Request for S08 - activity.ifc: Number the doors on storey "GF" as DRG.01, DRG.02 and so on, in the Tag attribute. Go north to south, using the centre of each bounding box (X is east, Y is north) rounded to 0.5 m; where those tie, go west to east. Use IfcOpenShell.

First a look at what the model holds.

```python
import ifcopenshell
import ifcopenshell.util.element
import ifcopenshell.util.placement

model = ifcopenshell.open("S08 - activity.ifc")
print(model.schema)
storey = next(s for s in model.by_type("IfcBuildingStorey") if s.Name == "GF")
doors = [e for e in ifcopenshell.util.element.get_decomposition(storey) if e.is_a("IfcDoor")]
for e in sorted(doors, key=lambda e: e.id()):
    origin = ifcopenshell.util.placement.get_local_placement(e.ObjectPlacement)[:3, 3]
    print(e.id(), e.Tag, e.Name, origin.round(2) + 0.0, sep=" | ")
```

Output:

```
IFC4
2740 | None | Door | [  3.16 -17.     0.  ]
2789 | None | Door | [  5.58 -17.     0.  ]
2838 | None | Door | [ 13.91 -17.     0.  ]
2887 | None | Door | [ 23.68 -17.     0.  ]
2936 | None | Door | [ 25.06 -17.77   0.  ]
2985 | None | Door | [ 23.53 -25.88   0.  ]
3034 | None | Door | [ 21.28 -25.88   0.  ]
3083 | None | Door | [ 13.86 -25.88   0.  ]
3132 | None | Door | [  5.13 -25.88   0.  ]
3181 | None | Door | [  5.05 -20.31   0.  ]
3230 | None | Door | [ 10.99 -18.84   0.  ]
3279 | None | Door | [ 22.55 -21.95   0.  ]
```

```python
import ifcopenshell
import ifcopenshell.geom
import ifcopenshell.util.element
import ifcopenshell.util.shape

model = ifcopenshell.open("S08 - activity.ifc")
settings = ifcopenshell.geom.settings()
settings.set("use-world-coords", True)


def centre(element):
    shape = ifcopenshell.geom.create_shape(settings, element)
    return ifcopenshell.util.shape.get_bbox_centroid(shape.geometry)


storey = next(s for s in model.by_type("IfcBuildingStorey") if s.Name == "GF")
doors = [e for e in ifcopenshell.util.element.get_decomposition(storey) if e.is_a("IfcDoor")]

# Insertion points can sit at a corner or the storey origin, so sort by the geometry (in metres).
centres = {e: centre(e) for e in doors}
doors.sort(key=lambda e: (-round(centres[e][1] / 0.5), centres[e][0]))

for i, e in enumerate(doors, start=1):
    number = f"DRG.{i:02d}"
    e.Tag = number
    print(e.id(), number)

model.write("S08 - activity_edited.ifc")
```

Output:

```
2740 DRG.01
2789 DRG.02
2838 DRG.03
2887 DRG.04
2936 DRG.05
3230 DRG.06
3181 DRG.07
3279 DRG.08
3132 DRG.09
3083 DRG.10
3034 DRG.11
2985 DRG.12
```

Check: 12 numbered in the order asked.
